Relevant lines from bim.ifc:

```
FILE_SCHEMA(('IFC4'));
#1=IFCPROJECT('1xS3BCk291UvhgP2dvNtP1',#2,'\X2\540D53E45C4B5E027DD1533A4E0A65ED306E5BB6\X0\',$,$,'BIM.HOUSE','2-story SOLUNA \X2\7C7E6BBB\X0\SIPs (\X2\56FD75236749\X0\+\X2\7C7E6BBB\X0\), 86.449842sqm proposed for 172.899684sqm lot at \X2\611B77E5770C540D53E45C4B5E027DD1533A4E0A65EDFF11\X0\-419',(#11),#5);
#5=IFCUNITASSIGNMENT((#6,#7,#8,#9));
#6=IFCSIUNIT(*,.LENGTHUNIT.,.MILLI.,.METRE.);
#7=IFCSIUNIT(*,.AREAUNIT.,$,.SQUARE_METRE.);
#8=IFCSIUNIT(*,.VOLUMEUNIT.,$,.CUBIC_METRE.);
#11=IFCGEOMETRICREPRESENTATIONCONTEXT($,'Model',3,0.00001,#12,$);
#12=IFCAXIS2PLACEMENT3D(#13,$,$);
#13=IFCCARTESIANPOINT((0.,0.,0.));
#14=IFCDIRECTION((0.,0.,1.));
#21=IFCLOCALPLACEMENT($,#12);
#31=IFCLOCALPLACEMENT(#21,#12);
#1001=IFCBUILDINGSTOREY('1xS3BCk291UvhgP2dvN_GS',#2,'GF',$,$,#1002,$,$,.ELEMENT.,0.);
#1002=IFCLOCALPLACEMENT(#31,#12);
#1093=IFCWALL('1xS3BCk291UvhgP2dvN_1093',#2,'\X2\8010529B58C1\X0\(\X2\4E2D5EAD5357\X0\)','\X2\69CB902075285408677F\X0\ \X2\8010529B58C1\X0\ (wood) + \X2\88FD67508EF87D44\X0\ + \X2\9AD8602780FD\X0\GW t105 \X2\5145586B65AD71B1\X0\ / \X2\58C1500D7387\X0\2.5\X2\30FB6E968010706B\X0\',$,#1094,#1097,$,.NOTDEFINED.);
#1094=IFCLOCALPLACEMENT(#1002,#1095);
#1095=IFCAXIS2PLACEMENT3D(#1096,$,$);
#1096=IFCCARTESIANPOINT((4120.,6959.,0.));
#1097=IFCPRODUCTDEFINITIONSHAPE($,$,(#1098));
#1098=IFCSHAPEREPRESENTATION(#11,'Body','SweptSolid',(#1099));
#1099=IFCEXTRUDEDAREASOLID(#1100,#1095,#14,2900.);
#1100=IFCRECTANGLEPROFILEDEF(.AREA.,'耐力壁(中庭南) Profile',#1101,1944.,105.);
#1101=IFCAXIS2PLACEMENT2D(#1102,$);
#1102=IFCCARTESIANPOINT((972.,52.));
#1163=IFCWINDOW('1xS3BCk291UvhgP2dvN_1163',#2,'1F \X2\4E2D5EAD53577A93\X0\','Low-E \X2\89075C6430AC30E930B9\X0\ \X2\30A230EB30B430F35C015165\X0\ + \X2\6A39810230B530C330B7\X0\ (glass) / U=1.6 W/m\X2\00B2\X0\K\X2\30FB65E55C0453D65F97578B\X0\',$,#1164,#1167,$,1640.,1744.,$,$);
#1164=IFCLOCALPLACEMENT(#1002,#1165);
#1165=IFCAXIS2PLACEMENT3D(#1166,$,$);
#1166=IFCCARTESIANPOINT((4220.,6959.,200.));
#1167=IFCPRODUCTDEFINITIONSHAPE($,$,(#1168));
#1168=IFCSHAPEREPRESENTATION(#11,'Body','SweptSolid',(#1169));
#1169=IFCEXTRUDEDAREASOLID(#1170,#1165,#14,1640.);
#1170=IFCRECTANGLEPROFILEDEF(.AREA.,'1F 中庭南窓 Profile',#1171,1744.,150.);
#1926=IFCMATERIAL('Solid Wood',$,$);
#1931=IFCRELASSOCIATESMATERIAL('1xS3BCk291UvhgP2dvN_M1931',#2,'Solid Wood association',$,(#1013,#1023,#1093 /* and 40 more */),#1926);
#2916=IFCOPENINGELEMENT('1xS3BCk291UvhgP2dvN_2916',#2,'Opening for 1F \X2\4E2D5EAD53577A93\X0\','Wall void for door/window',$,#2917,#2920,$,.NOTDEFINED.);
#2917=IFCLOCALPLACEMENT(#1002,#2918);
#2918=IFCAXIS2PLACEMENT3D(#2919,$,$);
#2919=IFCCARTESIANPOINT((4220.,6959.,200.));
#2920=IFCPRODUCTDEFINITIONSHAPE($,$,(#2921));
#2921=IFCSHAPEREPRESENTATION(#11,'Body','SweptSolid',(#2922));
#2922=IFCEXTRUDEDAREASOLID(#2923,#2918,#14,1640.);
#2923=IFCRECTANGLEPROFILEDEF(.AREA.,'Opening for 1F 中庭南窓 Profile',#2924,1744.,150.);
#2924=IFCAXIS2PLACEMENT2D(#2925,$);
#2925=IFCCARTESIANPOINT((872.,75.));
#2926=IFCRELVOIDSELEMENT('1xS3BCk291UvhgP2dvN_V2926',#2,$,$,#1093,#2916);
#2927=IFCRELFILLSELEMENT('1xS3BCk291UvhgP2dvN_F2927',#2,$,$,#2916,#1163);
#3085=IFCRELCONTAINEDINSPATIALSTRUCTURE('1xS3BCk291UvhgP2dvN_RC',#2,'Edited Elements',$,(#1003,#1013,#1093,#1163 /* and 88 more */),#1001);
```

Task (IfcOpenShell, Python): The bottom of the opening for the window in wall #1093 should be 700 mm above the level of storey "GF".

```python
import numpy as np
import ifcopenshell
import ifcopenshell.api.geometry
import ifcopenshell.geom
import ifcopenshell.util.element
import ifcopenshell.util.placement
import ifcopenshell.util.shape
import ifcopenshell.util.unit

model = ifcopenshell.open("bim.ifc")
unit_scale = ifcopenshell.util.unit.calculate_unit_scale(model)

window = model.by_guid("1xS3BCk291UvhgP2dvN_1163")
opening = window.FillsVoids[0].RelatingOpeningElement
storey = ifcopenshell.util.element.get_container(window, ifc_class="IfcBuildingStorey")
level = ifcopenshell.util.placement.get_local_placement(storey.ObjectPlacement)[2, 3]

# The opening's origin need not be at the sill, so measure its lowest point.
shape = ifcopenshell.geom.create_shape(ifcopenshell.geom.settings(), opening)
bottom = ifcopenshell.util.shape.get_shape_bottom_elevation(shape, shape.geometry) / unit_scale
dz = level + 0.7 / unit_scale - bottom

shift = np.array([0.0, 0.0, dz])
# The window is not placed relative to its opening, so move both.
for product in (opening, window):
    matrix = ifcopenshell.util.placement.get_local_placement(product.ObjectPlacement)
    matrix[:3, 3] += shift
    ifcopenshell.api.geometry.edit_object_placement(model, product=product, matrix=matrix, is_si=False)

print(f"moved by {dz * unit_scale:+.3f} m")

model.write("bim_updated.ifc")
```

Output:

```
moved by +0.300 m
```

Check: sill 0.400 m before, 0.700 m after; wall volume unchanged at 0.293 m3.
